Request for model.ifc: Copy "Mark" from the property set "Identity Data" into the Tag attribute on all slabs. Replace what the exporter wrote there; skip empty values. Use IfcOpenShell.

First a look at what the model holds.

```python
import ifcopenshell
import ifcopenshell.util.element

model = ifcopenshell.open("model.ifc")
print(model.schema)
slabs = model.by_type("IfcSlab")
print(len(slabs), "slabs")
for e in slabs[:8]:
    source = ifcopenshell.util.element.get_pset(e, "Identity Data", "Mark")
    target = e.Tag
    print(e.id(), repr(source), repr(target), sep=" | ")
```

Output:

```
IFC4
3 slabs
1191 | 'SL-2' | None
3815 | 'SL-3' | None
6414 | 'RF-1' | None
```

```python
import ifcopenshell
import ifcopenshell.util.element

model = ifcopenshell.open("model.ifc")

count = 0
for e in model.by_type("IfcSlab"):
    value = ifcopenshell.util.element.get_pset(e, "Identity Data", "Mark")
    current = e.Tag
    if not value or not value.strip() or current == value:
        continue
    e.Tag = value
    count += 1

print(count, "slabs updated")

model.write("model_rev.ifc")
```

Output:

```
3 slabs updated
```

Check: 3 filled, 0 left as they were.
